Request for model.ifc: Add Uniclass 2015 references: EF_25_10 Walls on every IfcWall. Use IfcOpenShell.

First a look at what the model holds.

```python
import ifcopenshell

model = ifcopenshell.open("model.ifc")
print(model.schema)
print("classifications:", [c.Name for c in model.by_type("IfcClassification")])
for ifc_class in ("IfcDoor", "IfcRoof", "IfcStair", "IfcWall", "IfcWindow"):
    print(ifc_class, len(model.by_type(ifc_class)))
```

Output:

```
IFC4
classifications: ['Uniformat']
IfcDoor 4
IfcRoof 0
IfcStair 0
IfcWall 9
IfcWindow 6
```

```python
import ifcopenshell
import ifcopenshell.api.classification

model = ifcopenshell.open("model.ifc")

system = ifcopenshell.api.classification.add_classification(model, classification="Uniclass 2015")

codes = {
    "IfcWall": ("EF_25_10", "Walls"),
}
for ifc_class, (code, name) in codes.items():
    products = model.by_type(ifc_class)
    ifcopenshell.api.classification.add_reference(
        model, products=products, classification=system, identification=code, name=name
    )
    print(code, len(products))

model.write("model_rev.ifc")
```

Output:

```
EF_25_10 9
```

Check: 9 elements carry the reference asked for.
